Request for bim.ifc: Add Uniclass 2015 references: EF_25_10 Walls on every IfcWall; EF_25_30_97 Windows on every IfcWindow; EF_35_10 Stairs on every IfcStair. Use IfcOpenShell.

First a look at what the model holds.

```python
import ifcopenshell

model = ifcopenshell.open("bim.ifc")
print(model.schema)
print("classifications:", [c.Name for c in model.by_type("IfcClassification")])
for ifc_class in ("IfcDoor", "IfcRoof", "IfcStair", "IfcWall", "IfcWindow"):
    print(ifc_class, len(model.by_type(ifc_class)))
```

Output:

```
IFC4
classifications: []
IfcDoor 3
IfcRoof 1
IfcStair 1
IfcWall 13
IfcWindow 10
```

```python
import ifcopenshell
import ifcopenshell.api.classification

model = ifcopenshell.open("bim.ifc")

system = ifcopenshell.api.classification.add_classification(model, classification="Uniclass 2015")

codes = {
    "IfcWall": ("EF_25_10", "Walls"),
    "IfcWindow": ("EF_25_30_97", "Windows"),
    "IfcStair": ("EF_35_10", "Stairs"),
}
for ifc_class, (code, name) in codes.items():
    products = model.by_type(ifc_class)
    ifcopenshell.api.classification.add_reference(
        model, products=products, classification=system, identification=code, name=name
    )
    print(code, len(products))

model.write("bim_rev.ifc")
```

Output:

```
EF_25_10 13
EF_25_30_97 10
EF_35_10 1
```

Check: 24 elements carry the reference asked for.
